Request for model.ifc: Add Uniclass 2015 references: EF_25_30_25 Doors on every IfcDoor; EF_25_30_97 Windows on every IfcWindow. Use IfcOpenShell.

First a look at what the model holds.

```python
import ifcopenshell

model = ifcopenshell.open("model.ifc")
print(model.schema)
print("classifications:", [c.Name for c in model.by_type("IfcClassification")])
for ifc_class in ("IfcDoor", "IfcRoof", "IfcStair", "IfcWall", "IfcWindow"):
    print(ifc_class, len(model.by_type(ifc_class)))
```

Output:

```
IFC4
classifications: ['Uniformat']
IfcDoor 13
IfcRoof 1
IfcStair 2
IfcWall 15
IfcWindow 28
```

```python
import ifcopenshell
import ifcopenshell.api.classification

model = ifcopenshell.open("model.ifc")

system = ifcopenshell.api.classification.add_classification(model, classification="Uniclass 2015")

codes = {
    "IfcDoor": ("EF_25_30_25", "Doors"),
    "IfcWindow": ("EF_25_30_97", "Windows"),
}
for ifc_class, (code, name) in codes.items():
    products = model.by_type(ifc_class)
    ifcopenshell.api.classification.add_reference(
        model, products=products, classification=system, identification=code, name=name
    )
    print(code, len(products))

model.write("model_v2.ifc")
```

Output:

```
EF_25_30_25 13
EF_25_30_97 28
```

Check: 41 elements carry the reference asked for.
